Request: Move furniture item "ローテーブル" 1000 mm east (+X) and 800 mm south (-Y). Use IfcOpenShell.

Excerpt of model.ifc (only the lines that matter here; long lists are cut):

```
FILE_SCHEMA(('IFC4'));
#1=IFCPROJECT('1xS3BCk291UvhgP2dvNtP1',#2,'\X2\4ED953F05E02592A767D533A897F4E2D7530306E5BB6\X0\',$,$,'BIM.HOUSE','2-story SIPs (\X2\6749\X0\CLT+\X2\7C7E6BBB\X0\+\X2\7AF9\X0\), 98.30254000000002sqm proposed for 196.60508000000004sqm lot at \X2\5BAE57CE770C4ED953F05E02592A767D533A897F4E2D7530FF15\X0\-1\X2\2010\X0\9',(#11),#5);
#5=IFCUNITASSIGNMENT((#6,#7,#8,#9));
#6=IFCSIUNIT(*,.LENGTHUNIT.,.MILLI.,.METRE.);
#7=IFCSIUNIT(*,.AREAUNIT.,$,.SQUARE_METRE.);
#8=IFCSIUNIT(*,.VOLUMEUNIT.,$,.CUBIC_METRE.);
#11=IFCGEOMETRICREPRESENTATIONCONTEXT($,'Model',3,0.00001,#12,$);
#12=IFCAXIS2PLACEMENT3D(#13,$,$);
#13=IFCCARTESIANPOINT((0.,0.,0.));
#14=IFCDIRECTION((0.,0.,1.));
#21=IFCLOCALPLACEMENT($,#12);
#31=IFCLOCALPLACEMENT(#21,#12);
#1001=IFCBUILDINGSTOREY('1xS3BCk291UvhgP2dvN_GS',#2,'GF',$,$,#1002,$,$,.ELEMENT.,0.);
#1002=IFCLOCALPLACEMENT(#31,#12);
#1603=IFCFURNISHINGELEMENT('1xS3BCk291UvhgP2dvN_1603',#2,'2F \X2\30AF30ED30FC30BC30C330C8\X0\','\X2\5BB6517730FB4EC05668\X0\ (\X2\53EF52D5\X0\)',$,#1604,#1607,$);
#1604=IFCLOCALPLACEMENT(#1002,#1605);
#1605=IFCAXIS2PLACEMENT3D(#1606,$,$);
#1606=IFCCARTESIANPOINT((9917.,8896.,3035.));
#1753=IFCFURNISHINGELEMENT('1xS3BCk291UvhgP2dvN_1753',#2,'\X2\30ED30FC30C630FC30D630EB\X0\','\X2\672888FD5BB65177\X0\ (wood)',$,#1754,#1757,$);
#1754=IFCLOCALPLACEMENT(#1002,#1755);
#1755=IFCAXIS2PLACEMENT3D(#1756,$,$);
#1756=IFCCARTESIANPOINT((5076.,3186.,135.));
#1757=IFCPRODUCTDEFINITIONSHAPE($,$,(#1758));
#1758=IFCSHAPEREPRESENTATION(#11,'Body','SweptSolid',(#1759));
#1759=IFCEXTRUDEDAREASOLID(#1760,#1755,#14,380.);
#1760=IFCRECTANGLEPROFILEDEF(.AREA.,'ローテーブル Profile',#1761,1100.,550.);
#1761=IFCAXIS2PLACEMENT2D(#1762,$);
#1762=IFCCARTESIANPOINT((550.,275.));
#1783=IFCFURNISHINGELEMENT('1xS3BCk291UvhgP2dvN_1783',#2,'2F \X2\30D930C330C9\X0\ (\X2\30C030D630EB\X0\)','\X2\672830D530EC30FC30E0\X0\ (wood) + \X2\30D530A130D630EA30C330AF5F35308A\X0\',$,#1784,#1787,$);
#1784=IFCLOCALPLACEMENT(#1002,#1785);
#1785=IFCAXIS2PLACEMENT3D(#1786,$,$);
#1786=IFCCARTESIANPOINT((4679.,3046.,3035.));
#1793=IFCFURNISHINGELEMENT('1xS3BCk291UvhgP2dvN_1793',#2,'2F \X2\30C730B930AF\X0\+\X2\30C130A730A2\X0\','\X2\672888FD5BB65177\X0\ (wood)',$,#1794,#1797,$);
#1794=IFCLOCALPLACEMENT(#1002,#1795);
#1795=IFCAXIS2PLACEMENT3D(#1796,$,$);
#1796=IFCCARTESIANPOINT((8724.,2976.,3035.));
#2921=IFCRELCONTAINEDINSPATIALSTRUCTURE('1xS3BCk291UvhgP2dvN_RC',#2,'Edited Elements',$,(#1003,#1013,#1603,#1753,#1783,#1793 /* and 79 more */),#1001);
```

```python
import ifcopenshell
import ifcopenshell.api.geometry
import ifcopenshell.util.placement
import ifcopenshell.util.unit

model = ifcopenshell.open("model.ifc")
unit_scale = ifcopenshell.util.unit.calculate_unit_scale(model)

item = model.by_guid("1xS3BCk291UvhgP2dvN_1753")
matrix = ifcopenshell.util.placement.get_local_placement(item.ObjectPlacement)
matrix[0, 3] += 1 / unit_scale
matrix[1, 3] -= 0.8 / unit_scale
ifcopenshell.api.geometry.edit_object_placement(model, product=item, matrix=matrix, is_si=False)

print(ifcopenshell.util.placement.get_local_placement(item.ObjectPlacement).round(3) + 0.0)

model.write("model_edited.ifc")
```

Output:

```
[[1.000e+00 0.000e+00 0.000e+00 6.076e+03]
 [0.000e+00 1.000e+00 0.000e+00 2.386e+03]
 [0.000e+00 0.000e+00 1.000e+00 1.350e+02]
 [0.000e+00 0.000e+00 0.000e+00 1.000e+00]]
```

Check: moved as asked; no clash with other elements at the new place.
